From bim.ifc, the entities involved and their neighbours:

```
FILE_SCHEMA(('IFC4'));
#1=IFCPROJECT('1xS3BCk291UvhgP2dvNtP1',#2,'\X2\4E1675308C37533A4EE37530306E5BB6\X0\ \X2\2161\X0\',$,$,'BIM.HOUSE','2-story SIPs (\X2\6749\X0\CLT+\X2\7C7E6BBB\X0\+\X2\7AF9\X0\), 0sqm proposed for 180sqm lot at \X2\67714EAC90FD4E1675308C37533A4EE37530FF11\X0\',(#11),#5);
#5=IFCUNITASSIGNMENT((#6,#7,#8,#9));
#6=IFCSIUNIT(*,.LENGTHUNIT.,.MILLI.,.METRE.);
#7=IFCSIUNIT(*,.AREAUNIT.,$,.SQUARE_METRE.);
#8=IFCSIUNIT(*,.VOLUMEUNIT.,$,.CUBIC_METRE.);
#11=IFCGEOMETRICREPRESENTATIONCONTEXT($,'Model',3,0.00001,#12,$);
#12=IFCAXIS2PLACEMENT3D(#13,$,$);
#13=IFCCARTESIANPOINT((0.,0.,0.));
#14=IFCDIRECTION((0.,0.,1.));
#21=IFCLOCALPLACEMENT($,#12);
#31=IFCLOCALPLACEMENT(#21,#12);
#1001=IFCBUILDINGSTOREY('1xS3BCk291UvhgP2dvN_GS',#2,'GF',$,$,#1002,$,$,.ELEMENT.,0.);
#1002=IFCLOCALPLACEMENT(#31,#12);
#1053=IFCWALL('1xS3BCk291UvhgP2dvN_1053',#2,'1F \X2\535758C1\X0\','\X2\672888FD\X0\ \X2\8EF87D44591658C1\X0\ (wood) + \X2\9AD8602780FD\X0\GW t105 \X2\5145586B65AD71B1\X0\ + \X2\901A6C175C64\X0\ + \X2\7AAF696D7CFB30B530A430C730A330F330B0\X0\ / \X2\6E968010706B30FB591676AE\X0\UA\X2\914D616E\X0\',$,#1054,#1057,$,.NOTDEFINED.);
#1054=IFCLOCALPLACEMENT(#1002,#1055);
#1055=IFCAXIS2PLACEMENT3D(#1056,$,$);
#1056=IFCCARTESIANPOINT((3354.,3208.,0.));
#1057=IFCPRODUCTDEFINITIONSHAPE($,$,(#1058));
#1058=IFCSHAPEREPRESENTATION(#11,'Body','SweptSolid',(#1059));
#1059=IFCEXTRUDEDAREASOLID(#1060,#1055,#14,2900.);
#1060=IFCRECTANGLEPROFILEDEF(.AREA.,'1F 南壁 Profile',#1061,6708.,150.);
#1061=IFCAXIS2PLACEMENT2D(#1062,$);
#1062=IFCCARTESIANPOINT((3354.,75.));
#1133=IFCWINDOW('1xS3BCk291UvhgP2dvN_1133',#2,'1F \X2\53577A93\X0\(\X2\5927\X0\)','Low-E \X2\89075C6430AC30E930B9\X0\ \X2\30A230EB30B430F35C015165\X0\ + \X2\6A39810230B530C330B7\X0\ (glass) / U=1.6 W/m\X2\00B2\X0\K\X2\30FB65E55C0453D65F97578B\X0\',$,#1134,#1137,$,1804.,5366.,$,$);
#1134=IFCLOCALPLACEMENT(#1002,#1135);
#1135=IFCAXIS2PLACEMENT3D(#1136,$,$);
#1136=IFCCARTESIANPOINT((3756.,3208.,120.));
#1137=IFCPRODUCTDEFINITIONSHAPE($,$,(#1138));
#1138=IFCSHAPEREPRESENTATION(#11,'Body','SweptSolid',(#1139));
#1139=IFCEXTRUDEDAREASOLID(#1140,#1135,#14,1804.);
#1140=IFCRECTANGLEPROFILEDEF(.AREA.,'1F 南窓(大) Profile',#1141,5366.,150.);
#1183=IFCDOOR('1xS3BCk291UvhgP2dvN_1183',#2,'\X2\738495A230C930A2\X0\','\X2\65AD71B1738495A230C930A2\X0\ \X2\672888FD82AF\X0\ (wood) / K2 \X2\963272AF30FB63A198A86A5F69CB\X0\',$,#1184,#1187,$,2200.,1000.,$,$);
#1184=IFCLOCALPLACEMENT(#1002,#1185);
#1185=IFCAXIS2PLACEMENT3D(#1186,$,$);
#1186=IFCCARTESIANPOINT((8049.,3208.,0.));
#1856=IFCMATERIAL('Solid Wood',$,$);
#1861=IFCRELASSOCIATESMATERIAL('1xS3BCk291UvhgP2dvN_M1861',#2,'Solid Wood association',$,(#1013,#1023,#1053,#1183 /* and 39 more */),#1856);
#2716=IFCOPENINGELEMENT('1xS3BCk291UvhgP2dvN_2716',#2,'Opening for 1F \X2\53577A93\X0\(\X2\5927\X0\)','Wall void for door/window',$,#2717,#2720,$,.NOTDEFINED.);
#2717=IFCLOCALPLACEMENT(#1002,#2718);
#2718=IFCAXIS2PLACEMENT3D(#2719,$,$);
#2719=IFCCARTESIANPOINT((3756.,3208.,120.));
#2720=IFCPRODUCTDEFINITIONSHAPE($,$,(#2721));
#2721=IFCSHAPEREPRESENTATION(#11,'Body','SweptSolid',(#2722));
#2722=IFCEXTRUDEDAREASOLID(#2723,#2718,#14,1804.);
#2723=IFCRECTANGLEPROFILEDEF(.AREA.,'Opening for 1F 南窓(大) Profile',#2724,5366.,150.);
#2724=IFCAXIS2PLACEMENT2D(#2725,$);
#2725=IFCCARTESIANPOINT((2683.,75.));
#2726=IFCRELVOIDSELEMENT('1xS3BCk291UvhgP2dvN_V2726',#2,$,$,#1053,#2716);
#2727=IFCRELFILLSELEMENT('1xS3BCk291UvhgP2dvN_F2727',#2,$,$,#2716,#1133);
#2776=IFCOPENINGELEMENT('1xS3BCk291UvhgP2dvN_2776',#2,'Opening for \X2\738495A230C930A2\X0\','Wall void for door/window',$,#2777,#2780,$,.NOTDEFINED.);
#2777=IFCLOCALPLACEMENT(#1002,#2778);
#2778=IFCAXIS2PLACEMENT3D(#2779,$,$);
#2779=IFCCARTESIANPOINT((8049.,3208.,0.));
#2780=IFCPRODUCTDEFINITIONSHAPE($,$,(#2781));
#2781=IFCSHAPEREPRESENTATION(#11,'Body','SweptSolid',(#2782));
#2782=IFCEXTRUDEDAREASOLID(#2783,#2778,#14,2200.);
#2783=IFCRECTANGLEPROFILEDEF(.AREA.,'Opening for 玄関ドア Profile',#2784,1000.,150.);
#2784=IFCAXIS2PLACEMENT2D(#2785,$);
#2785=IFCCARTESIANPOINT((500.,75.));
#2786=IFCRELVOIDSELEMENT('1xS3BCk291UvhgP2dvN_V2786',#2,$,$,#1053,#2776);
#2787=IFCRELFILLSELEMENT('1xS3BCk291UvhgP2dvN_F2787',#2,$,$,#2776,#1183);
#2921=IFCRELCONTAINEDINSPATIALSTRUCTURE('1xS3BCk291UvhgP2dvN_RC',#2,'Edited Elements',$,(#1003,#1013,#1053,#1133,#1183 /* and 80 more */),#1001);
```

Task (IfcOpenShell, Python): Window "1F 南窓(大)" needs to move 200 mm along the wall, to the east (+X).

```python
import ifcopenshell
import ifcopenshell.api.geometry
import ifcopenshell.util.placement
import ifcopenshell.util.unit

model = ifcopenshell.open("bim.ifc")
unit_scale = ifcopenshell.util.unit.calculate_unit_scale(model)

window = model.by_guid("1xS3BCk291UvhgP2dvN_1133")
opening = window.FillsVoids[0].RelatingOpeningElement
wall = opening.VoidsElements[0].RelatingBuildingElement

wall_matrix = ifcopenshell.util.placement.get_local_placement(wall.ObjectPlacement)
shift = wall_matrix[:3, 0] * 0.2 / unit_scale
before = ifcopenshell.util.placement.get_local_placement(window.ObjectPlacement)[:3, 3].copy()

# The window is not placed relative to its opening, so move both.
for product in (opening, window):
    matrix = ifcopenshell.util.placement.get_local_placement(product.ObjectPlacement)
    matrix[:3, 3] += shift
    ifcopenshell.api.geometry.edit_object_placement(model, product=product, matrix=matrix, is_si=False)

after = ifcopenshell.util.placement.get_local_placement(window.ObjectPlacement)[:3, 3]
print("window moved by", (after - before).round(3) + 0.0)

model.write("bim_v2.ifc")
```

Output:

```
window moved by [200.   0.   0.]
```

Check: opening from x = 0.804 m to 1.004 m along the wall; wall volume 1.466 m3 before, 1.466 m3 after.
